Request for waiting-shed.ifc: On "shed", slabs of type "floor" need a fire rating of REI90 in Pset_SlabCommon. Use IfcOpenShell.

First a look at what the model holds.

```python
import ifcopenshell
import ifcopenshell.util.element

model = ifcopenshell.open("waiting-shed.ifc")
print(model.schema)
storey = next(s for s in model.by_type("IfcBuildingStorey") if s.Name == "shed")
slabs = [e for e in ifcopenshell.util.element.get_decomposition(storey) if e.is_a("IfcSlab")]
seen = {}
for e in slabs:
    element_type = ifcopenshell.util.element.get_type(e)
    key = (element_type.Name if element_type != e and element_type else None, ifcopenshell.util.element.get_pset(e, "Pset_SlabCommon", "FireRating"))
    seen[key] = seen.get(key, 0) + 1
for (name, value), count in sorted(seen.items(), key=str):
    print(count, "x", name, "|", value)
```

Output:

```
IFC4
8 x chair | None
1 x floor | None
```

```python
import ifcopenshell
import ifcopenshell.api.pset
import ifcopenshell.util.element

model = ifcopenshell.open("waiting-shed.ifc")

storey = next(s for s in model.by_type("IfcBuildingStorey") if s.Name == "shed")
slabs = [e for e in ifcopenshell.util.element.get_decomposition(storey) if e.is_a("IfcSlab")]

count = 0
for e in slabs:
    element_type = ifcopenshell.util.element.get_type(e)
    if element_type in (None, e) or element_type.Name != "floor":
        continue
    # add_pset returns the element's existing set when there is one.
    pset = ifcopenshell.api.pset.add_pset(model, product=e, name="Pset_SlabCommon")
    ifcopenshell.api.pset.edit_pset(model, pset=pset, properties={"FireRating": "REI90"})
    count += 1

print(count, "slabs updated")

model.write("waiting-shed_edited.ifc")
```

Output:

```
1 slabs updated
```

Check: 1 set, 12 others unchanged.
